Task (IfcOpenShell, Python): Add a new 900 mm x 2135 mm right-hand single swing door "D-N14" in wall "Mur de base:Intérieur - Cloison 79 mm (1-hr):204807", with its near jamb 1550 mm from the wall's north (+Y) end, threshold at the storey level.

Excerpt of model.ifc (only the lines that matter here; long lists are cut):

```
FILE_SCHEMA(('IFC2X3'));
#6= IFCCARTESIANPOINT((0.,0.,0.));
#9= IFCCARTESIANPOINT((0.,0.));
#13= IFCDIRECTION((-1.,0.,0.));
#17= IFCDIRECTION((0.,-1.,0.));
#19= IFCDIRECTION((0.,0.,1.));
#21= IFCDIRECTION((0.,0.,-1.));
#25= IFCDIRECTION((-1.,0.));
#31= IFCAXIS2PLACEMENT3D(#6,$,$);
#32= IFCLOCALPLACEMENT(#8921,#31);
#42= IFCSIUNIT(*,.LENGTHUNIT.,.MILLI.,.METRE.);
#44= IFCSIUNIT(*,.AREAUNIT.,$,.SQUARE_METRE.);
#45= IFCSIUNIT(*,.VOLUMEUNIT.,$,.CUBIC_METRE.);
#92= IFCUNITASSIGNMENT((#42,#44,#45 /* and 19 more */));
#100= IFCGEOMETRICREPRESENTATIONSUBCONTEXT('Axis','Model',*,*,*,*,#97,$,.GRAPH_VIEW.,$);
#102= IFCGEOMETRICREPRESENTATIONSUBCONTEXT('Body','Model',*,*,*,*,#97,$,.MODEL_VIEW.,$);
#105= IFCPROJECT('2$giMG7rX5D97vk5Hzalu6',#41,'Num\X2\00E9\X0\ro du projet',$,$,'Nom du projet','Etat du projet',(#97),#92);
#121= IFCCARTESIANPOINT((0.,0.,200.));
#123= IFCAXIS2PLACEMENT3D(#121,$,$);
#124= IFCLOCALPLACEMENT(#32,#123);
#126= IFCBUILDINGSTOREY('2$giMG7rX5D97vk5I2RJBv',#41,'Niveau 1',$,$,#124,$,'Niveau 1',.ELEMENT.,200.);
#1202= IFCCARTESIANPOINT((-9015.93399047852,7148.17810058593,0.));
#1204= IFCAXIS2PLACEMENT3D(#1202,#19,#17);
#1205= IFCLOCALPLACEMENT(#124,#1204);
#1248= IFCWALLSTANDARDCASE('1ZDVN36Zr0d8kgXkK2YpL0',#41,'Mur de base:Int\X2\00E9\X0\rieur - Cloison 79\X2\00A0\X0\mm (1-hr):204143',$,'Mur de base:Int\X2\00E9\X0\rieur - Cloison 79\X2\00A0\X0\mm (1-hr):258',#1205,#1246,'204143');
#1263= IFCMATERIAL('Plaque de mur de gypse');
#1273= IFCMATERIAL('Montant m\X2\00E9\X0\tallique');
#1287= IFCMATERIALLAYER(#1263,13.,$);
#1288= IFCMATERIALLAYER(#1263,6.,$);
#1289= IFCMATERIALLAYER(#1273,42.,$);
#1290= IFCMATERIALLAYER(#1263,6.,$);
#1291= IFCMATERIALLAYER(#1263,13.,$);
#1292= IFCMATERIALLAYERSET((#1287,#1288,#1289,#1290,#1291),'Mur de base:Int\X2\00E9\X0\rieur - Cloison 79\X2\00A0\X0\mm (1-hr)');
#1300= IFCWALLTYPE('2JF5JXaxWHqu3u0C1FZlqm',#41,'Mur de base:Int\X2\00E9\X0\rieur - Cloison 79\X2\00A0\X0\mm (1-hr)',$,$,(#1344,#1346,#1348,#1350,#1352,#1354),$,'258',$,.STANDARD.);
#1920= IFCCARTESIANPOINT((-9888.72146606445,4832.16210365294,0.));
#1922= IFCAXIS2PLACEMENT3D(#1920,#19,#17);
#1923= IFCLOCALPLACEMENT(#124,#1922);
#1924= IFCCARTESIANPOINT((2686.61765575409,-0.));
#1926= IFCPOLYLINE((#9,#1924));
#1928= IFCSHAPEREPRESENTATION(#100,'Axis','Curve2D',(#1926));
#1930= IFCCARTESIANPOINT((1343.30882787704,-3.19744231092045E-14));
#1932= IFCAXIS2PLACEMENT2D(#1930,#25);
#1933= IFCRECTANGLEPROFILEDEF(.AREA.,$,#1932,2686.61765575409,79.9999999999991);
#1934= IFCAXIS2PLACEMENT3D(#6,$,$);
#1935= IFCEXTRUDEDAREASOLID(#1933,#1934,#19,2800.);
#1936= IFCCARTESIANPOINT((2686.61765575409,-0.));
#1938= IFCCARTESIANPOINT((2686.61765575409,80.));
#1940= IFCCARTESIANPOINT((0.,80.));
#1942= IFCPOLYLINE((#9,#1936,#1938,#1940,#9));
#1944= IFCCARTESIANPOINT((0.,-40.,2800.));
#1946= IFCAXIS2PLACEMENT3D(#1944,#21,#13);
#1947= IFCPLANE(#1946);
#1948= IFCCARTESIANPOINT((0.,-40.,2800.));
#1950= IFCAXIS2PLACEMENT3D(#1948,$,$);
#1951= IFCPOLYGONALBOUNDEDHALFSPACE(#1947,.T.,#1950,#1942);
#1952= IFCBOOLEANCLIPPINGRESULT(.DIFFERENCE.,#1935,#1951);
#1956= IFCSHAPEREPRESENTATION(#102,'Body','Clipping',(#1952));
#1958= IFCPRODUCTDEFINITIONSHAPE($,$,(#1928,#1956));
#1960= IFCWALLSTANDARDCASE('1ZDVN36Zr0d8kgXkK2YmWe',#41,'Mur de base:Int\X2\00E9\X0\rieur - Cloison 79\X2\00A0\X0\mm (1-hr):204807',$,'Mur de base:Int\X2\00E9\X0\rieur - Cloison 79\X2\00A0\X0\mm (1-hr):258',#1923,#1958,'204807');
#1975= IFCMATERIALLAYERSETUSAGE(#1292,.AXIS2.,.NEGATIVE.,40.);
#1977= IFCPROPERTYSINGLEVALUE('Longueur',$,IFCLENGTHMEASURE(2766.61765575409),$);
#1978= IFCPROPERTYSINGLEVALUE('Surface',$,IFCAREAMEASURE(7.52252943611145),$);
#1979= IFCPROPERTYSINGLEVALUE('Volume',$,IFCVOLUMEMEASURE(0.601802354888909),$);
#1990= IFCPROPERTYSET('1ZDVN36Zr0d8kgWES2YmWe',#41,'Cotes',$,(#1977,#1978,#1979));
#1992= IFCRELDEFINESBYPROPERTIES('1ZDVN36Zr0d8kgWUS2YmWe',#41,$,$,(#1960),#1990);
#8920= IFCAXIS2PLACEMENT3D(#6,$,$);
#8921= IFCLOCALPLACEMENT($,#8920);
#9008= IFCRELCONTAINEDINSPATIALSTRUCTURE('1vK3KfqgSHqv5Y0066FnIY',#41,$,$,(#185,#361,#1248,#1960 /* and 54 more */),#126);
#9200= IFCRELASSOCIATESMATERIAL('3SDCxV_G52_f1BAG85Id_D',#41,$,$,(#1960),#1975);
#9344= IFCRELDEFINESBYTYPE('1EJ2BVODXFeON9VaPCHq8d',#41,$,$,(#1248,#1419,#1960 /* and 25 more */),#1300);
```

```python
import numpy as np
import ifcopenshell
import ifcopenshell.api.feature
import ifcopenshell.api.geometry
import ifcopenshell.api.pset
import ifcopenshell.api.root
import ifcopenshell.api.spatial
import ifcopenshell.api.type
import ifcopenshell.geom
import ifcopenshell.util.element
import ifcopenshell.util.placement
import ifcopenshell.util.representation
import ifcopenshell.util.shape
import ifcopenshell.util.unit

model = ifcopenshell.open("model.ifc")
unit_scale = ifcopenshell.util.unit.calculate_unit_scale(model)
area_scale = ifcopenshell.util.unit.calculate_unit_scale(model, "AREAUNIT")
volume_scale = ifcopenshell.util.unit.calculate_unit_scale(model, "VOLUMEUNIT")
settings = ifcopenshell.geom.settings()


def volume(element):
    """Net volume in cubic metres, openings subtracted."""
    shape = ifcopenshell.geom.create_shape(settings, element)
    return ifcopenshell.util.shape.get_volume(shape.geometry)


wall = model.by_guid("1ZDVN36Zr0d8kgXkK2YmWe")
storey = ifcopenshell.util.element.get_container(wall, ifc_class="IfcBuildingStorey")
context = ifcopenshell.util.representation.get_context(model, "Model", "Body", "MODEL_VIEW")
before = volume(wall)

width, height, from_end, sill = 0.9, 2.135, 1.55, 0.0  # metres

# The wall runs along its own X axis, and the end named is its -X end.
wall_shape = ifcopenshell.geom.create_shape(settings, wall)
x, y, z = ifcopenshell.util.shape.get_vertices(wall_shape.geometry).T
start = x.min() + from_end
face, thickness = float(y.min()), float(y.max() - y.min())
wall_matrix = ifcopenshell.util.placement.get_local_placement(wall.ObjectPlacement)
level = ifcopenshell.util.placement.get_local_placement(storey.ObjectPlacement)[2, 3]


def in_wall(x, y):
    """Placement at x, y metres in the wall's axes, at sill height."""
    matrix = wall_matrix.copy()
    matrix[:, 3] = wall_matrix @ np.array([x / unit_scale, y / unit_scale, 0.0, 1.0])
    matrix[2, 3] = level + sill / unit_scale
    return matrix


# Opening: a box that overshoots both wall faces by 50 mm.
opening = ifcopenshell.api.root.create_entity(model, ifc_class="IfcOpeningElement")
box = ifcopenshell.api.geometry.add_wall_representation(
    model, context=context, length=width, height=height, thickness=thickness + 0.1
)
ifcopenshell.api.geometry.assign_representation(model, product=opening, representation=box)
ifcopenshell.api.geometry.edit_object_placement(model, product=opening, matrix=in_wall(start, face - 0.05), is_si=False)
ifcopenshell.api.feature.add_feature(model, feature=opening, element=wall)

door = ifcopenshell.api.root.create_entity(model, ifc_class="IfcDoor", name="D-N14")
door.OverallWidth, door.OverallHeight = width / unit_scale, height / unit_scale
body = ifcopenshell.api.geometry.add_door_representation(
    model,
    context=context,
    overall_width=door.OverallWidth,
    overall_height=door.OverallHeight,
    operation_type="SINGLE_SWING_RIGHT",
    lining_properties={"LiningDepth": thickness / unit_scale, "ThresholdDepth": thickness / unit_scale},
)
ifcopenshell.api.geometry.assign_representation(model, product=door, representation=body)
ifcopenshell.api.spatial.assign_container(model, products=[door], relating_structure=storey)
fills = ifcopenshell.api.feature.add_filling(model, opening=opening, element=door)
fills.OwnerHistory = door.OwnerHistory  # required in IFC2X3

# IFC2X3 keeps the operation on the door style.
style = ifcopenshell.api.root.create_entity(model, ifc_class="IfcDoorStyle", name="D-N14")
style.OperationType, style.ConstructionType = "SINGLE_SWING_RIGHT", "NOTDEFINED"
style.ParameterTakesPrecedence = style.Sizeable = False
ifcopenshell.api.type.assign_type(model, related_objects=[door], relating_type=style)

# The lining spans the wall, so the door starts at the wall face.
ifcopenshell.api.geometry.edit_object_placement(model, product=door, matrix=in_wall(start, face), is_si=False)

after = volume(wall)

# Update the wall's stored quantities.
pset = model.by_id(ifcopenshell.util.element.get_pset(wall, "Cotes", should_inherit=False)["id"])
ifcopenshell.api.pset.edit_pset(model, pset=pset, properties={
    "Surface": model.create_entity("IfcAreaMeasure", after / thickness / area_scale),
    "Volume": model.create_entity("IfcVolumeMeasure", after / volume_scale),
})

print(f"wall volume {before:.3f} -> {after:.3f} m3")

model.write("model_v2.ifc")
```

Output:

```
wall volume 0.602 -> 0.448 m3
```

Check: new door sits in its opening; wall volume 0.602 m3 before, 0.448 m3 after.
